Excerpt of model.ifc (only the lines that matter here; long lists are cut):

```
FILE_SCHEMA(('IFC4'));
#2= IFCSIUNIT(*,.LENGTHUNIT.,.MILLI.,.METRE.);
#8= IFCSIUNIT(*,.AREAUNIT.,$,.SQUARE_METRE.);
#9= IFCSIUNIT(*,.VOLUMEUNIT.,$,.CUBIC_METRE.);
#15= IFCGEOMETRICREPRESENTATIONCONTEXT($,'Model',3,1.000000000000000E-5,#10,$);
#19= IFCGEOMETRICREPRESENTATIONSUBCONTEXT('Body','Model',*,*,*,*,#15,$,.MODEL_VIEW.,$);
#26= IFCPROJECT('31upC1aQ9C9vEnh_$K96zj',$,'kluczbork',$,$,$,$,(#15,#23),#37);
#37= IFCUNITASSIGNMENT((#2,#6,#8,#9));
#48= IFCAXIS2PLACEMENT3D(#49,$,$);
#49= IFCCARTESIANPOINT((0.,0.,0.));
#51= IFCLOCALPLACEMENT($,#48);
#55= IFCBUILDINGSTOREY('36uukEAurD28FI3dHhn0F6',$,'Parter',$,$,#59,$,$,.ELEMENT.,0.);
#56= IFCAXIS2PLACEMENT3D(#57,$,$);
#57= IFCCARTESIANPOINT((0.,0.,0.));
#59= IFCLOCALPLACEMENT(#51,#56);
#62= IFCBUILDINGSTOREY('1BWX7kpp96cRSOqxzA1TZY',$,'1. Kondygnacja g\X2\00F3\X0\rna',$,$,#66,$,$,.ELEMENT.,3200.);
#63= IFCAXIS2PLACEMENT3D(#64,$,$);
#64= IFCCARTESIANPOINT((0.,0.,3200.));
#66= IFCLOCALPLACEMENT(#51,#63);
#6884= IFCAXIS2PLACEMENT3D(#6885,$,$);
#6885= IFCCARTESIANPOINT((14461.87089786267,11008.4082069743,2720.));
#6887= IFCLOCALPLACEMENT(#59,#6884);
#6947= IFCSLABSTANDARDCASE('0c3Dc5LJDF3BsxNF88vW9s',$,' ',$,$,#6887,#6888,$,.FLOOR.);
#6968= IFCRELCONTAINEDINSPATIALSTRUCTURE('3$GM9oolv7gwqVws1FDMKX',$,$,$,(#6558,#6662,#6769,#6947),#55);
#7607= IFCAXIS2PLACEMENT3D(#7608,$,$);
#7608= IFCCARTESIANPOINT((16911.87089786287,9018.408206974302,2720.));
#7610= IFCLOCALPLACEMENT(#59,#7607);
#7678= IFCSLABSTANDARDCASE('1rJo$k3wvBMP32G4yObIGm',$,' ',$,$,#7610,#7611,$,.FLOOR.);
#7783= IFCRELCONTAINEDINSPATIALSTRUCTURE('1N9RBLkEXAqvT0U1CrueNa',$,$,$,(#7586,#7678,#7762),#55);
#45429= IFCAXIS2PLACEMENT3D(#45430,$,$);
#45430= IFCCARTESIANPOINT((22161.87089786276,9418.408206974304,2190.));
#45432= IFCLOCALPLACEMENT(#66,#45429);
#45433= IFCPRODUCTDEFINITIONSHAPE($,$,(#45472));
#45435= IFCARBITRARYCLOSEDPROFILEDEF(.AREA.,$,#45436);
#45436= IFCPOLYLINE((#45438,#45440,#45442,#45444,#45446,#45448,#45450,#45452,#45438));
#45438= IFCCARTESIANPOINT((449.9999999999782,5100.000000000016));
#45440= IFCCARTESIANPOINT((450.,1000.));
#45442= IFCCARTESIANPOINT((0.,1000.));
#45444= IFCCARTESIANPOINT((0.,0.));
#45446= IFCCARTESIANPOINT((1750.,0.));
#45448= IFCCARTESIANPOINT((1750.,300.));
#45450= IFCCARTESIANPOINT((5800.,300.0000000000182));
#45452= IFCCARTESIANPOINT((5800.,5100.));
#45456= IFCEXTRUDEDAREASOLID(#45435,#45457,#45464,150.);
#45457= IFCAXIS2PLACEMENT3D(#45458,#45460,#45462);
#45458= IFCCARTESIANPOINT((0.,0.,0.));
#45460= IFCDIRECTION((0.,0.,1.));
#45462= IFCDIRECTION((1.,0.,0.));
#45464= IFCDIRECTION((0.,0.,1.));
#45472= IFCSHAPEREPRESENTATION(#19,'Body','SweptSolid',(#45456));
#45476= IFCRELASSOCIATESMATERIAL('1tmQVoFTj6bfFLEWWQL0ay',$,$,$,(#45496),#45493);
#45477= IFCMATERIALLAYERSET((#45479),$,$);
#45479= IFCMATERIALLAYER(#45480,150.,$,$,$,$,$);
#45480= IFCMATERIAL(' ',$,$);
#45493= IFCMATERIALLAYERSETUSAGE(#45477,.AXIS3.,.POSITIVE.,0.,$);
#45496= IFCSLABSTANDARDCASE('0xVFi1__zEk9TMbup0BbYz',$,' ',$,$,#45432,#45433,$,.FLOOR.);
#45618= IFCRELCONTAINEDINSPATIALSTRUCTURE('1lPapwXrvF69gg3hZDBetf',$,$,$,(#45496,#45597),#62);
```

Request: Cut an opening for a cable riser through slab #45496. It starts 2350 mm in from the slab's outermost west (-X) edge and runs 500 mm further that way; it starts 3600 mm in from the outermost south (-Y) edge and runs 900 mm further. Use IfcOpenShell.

```python
import numpy as np
import ifcopenshell
import ifcopenshell.api.feature
import ifcopenshell.api.geometry
import ifcopenshell.api.root
import ifcopenshell.geom
import ifcopenshell.util.placement
import ifcopenshell.util.representation
import ifcopenshell.util.shape
import ifcopenshell.util.unit

model = ifcopenshell.open("model.ifc")
unit_scale = ifcopenshell.util.unit.calculate_unit_scale(model)
settings = ifcopenshell.geom.settings()


def volume(element):
    """Net volume in cubic metres, openings subtracted."""
    shape = ifcopenshell.geom.create_shape(settings, element)
    return ifcopenshell.util.shape.get_volume(shape.geometry)


slab = model.by_guid("0xVFi1__zEk9TMbup0BbYz")
before = volume(slab)

# Extent in the slab's own axes, in metres. The edges named are its -X and -Y sides.
slab_shape = ifcopenshell.geom.create_shape(settings, slab)
vertices = ifcopenshell.util.shape.get_vertices(slab_shape.geometry)
x_min, y_min, bottom = vertices.min(axis=0)
top = vertices[:, 2].max()

opening = ifcopenshell.api.root.create_entity(model, ifc_class="IfcOpeningElement", name="Cable riser opening", predefined_type="OPENING")
context = ifcopenshell.util.representation.get_context(model, "Model", "Body", "MODEL_VIEW")
width, depth = 0.5, 0.9
outline = [(0.0, 0.0), (width, 0.0), (width, depth), (0.0, depth), (0.0, 0.0)]
# Overshoot both faces by 50 mm so the cut is clean.
shape = ifcopenshell.api.geometry.add_slab_representation(
    model, context=context, depth=top - bottom + 0.1, polyline=outline
)
ifcopenshell.api.geometry.assign_representation(model, product=opening, representation=shape)

matrix = ifcopenshell.util.placement.get_local_placement(slab.ObjectPlacement)
matrix[:, 3] = matrix @ np.append(np.array([x_min + 2.35, y_min + 3.6, bottom - 0.05]) / unit_scale, 1.0)
ifcopenshell.api.geometry.edit_object_placement(model, product=opening, matrix=matrix, is_si=False)
ifcopenshell.api.feature.add_feature(model, feature=opening, element=slab)

after = volume(slab)

print(f"slab volume {before:.3f} -> {after:.3f} m3")

model.write("model_rev.ifc")
```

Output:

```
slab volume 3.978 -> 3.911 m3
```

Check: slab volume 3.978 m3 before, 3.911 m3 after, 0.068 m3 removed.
